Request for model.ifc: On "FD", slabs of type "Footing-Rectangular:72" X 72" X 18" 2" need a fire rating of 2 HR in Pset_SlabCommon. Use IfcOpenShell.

First a look at what the model holds.

```python
import ifcopenshell
import ifcopenshell.util.element

model = ifcopenshell.open("model.ifc")
print(model.schema)
storey = next(s for s in model.by_type("IfcBuildingStorey") if s.Name == "FD")
slabs = [e for e in ifcopenshell.util.element.get_decomposition(storey) if e.is_a("IfcSlab")]
seen = {}
for e in slabs:
    element_type = ifcopenshell.util.element.get_type(e)
    key = (element_type.Name if element_type != e and element_type else None, ifcopenshell.util.element.get_pset(e, "Pset_SlabCommon", "FireRating"))
    seen[key] = seen.get(key, 0) + 1
for (name, value), count in sorted(seen.items(), key=str):
    print(count, "x", name, "|", value)
```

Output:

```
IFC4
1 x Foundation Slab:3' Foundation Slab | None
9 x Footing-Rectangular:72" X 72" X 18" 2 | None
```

```python
import ifcopenshell
import ifcopenshell.api.pset
import ifcopenshell.util.element

model = ifcopenshell.open("model.ifc")

storey = next(s for s in model.by_type("IfcBuildingStorey") if s.Name == "FD")
slabs = [e for e in ifcopenshell.util.element.get_decomposition(storey) if e.is_a("IfcSlab")]

count = 0
for e in slabs:
    element_type = ifcopenshell.util.element.get_type(e)
    if element_type in (None, e) or element_type.Name != 'Footing-Rectangular:72" X 72" X 18" 2':
        continue
    # add_pset returns the element's existing set when there is one.
    pset = ifcopenshell.api.pset.add_pset(model, product=e, name="Pset_SlabCommon")
    ifcopenshell.api.pset.edit_pset(model, pset=pset, properties={"FireRating": "2 HR"})
    count += 1

print(count, "slabs updated")

model.write("model_rev.ifc")
```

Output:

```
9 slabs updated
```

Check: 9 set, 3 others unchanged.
